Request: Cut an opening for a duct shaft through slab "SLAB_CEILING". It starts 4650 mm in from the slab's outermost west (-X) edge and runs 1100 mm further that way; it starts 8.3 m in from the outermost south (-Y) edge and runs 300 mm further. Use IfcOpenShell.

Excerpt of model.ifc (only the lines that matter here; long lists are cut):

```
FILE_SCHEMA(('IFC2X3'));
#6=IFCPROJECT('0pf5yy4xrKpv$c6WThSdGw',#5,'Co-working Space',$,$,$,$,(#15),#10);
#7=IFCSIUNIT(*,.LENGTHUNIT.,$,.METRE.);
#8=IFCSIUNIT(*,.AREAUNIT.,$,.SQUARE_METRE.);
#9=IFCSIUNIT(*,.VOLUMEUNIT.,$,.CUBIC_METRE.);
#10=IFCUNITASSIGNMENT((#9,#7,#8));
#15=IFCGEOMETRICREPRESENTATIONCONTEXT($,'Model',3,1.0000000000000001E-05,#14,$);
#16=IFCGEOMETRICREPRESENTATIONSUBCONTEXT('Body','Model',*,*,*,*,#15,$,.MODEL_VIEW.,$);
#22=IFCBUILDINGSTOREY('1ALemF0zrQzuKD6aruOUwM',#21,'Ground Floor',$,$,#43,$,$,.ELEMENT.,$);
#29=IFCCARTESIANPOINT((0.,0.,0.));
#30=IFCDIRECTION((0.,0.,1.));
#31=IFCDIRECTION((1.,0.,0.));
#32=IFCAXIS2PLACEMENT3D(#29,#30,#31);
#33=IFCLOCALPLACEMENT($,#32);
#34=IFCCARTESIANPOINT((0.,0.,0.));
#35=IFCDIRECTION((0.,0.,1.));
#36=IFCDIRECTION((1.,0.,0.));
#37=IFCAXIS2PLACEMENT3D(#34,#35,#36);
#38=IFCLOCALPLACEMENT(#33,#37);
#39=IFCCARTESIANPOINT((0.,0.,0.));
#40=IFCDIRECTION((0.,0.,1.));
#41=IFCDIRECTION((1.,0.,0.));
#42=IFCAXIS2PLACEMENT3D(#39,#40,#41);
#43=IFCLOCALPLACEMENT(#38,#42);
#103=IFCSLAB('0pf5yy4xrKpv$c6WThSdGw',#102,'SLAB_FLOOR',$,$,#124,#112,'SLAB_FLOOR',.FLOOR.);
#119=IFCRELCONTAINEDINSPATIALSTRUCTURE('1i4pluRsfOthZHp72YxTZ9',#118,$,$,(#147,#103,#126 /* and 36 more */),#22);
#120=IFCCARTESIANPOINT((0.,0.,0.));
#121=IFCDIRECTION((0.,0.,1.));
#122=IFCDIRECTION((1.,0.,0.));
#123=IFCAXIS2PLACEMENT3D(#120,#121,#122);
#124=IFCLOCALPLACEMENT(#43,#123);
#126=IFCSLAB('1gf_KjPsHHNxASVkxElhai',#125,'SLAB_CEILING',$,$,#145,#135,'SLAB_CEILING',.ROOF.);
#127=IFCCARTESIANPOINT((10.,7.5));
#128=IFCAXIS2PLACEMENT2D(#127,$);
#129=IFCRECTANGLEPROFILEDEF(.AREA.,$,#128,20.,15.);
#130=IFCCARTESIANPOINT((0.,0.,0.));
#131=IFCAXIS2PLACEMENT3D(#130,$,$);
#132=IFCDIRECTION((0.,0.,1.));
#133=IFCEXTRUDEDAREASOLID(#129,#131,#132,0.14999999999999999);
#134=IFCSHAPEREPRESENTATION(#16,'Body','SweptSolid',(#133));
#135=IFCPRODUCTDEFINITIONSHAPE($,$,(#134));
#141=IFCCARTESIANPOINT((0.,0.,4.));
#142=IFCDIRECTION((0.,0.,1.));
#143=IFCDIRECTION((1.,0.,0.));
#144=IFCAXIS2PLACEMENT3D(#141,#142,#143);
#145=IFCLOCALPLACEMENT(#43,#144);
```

```python
import numpy as np
import ifcopenshell
import ifcopenshell.api.feature
import ifcopenshell.api.geometry
import ifcopenshell.api.root
import ifcopenshell.geom
import ifcopenshell.util.placement
import ifcopenshell.util.representation
import ifcopenshell.util.shape
import ifcopenshell.util.unit

model = ifcopenshell.open("model.ifc")
unit_scale = ifcopenshell.util.unit.calculate_unit_scale(model)
settings = ifcopenshell.geom.settings()


def volume(element):
    """Net volume in cubic metres, openings subtracted."""
    shape = ifcopenshell.geom.create_shape(settings, element)
    return ifcopenshell.util.shape.get_volume(shape.geometry)


slab = model.by_id(126)
before = volume(slab)

# Extent in the slab's own axes, in metres. The edges named are its -X and -Y sides.
slab_shape = ifcopenshell.geom.create_shape(settings, slab)
vertices = ifcopenshell.util.shape.get_vertices(slab_shape.geometry)
x_min, y_min, bottom = vertices.min(axis=0)
top = vertices[:, 2].max()

opening = ifcopenshell.api.root.create_entity(model, ifc_class="IfcOpeningElement", name="Duct shaft opening")
context = ifcopenshell.util.representation.get_context(model, "Model", "Body", "MODEL_VIEW")
width, depth = 1.1, 0.3
outline = [(0.0, 0.0), (width, 0.0), (width, depth), (0.0, depth), (0.0, 0.0)]
# Overshoot both faces by 50 mm so the cut is clean.
shape = ifcopenshell.api.geometry.add_slab_representation(
    model, context=context, depth=top - bottom + 0.1, polyline=outline
)
ifcopenshell.api.geometry.assign_representation(model, product=opening, representation=shape)

matrix = ifcopenshell.util.placement.get_local_placement(slab.ObjectPlacement)
matrix[:, 3] = matrix @ np.append(np.array([x_min + 4.65, y_min + 8.3, bottom - 0.05]) / unit_scale, 1.0)
ifcopenshell.api.geometry.edit_object_placement(model, product=opening, matrix=matrix, is_si=False)
ifcopenshell.api.feature.add_feature(model, feature=opening, element=slab)

after = volume(slab)

print(f"slab volume {before:.3f} -> {after:.3f} m3")

model.write("model-out.ifc")
```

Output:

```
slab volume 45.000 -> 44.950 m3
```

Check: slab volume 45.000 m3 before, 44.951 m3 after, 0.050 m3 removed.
